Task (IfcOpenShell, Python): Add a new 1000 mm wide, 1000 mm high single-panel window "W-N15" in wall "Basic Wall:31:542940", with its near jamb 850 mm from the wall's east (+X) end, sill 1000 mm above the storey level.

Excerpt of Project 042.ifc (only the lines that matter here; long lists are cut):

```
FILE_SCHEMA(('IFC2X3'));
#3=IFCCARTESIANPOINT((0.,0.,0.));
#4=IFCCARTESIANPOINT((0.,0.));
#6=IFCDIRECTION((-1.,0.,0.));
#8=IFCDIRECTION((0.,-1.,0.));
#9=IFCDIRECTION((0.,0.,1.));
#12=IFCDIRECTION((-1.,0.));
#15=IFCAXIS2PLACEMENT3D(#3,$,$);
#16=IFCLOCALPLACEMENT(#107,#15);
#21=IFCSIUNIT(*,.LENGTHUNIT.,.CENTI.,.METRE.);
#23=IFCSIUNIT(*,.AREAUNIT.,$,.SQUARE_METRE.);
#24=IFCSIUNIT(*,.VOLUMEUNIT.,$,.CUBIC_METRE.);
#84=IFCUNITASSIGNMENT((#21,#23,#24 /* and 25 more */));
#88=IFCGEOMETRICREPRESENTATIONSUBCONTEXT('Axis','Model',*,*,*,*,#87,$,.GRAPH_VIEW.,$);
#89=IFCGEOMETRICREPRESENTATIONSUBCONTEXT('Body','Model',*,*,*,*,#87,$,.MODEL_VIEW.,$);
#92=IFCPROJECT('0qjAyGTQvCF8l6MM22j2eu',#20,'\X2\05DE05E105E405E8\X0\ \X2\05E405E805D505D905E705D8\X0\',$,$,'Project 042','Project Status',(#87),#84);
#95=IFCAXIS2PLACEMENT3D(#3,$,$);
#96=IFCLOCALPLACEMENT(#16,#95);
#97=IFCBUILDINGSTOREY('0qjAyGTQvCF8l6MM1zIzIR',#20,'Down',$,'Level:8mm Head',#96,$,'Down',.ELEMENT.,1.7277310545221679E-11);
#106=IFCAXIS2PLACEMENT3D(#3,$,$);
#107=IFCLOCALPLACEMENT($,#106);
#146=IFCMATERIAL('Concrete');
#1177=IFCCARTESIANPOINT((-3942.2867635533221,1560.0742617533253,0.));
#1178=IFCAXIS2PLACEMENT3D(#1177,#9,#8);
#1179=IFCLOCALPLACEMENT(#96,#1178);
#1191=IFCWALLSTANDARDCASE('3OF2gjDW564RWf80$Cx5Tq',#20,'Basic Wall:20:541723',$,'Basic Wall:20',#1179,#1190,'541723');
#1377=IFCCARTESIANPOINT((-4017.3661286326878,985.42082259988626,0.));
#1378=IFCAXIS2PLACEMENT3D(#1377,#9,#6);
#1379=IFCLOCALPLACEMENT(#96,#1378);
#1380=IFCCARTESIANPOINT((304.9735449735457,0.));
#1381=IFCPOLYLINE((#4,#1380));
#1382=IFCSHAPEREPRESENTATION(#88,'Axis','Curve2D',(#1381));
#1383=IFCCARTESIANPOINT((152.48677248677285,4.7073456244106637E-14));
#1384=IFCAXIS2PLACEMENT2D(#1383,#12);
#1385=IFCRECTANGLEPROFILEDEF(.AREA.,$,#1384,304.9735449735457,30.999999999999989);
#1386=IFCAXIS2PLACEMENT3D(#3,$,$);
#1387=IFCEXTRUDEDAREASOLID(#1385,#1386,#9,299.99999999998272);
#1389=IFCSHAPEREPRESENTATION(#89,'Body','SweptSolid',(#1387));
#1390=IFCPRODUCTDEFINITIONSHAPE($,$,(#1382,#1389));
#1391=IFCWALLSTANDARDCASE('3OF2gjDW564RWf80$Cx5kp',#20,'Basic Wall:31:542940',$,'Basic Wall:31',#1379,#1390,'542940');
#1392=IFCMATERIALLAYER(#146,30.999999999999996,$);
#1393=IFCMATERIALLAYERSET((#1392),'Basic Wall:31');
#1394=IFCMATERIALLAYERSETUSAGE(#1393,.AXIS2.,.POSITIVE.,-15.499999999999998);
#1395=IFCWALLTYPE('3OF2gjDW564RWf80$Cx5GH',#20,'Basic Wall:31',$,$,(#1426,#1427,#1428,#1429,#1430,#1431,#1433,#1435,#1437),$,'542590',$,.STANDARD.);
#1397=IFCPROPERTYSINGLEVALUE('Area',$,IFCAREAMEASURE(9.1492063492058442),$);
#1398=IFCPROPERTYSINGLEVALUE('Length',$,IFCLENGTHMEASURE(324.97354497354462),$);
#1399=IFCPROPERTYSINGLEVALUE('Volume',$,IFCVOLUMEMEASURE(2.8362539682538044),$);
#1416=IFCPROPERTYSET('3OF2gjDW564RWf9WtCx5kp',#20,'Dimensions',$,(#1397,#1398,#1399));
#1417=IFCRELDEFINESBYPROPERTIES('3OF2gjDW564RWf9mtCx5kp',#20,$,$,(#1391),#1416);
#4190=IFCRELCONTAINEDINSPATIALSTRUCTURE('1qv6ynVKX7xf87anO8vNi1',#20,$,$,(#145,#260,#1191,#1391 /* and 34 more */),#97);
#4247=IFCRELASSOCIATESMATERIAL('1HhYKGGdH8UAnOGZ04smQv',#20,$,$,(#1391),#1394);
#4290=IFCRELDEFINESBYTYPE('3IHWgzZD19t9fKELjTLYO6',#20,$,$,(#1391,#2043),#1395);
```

```python
import numpy as np
import ifcopenshell
import ifcopenshell.api.feature
import ifcopenshell.api.geometry
import ifcopenshell.api.pset
import ifcopenshell.api.root
import ifcopenshell.api.spatial
import ifcopenshell.api.type
import ifcopenshell.geom
import ifcopenshell.util.element
import ifcopenshell.util.placement
import ifcopenshell.util.representation
import ifcopenshell.util.shape
import ifcopenshell.util.unit

model = ifcopenshell.open("Project 042.ifc")
unit_scale = ifcopenshell.util.unit.calculate_unit_scale(model)
area_scale = ifcopenshell.util.unit.calculate_unit_scale(model, "AREAUNIT")
volume_scale = ifcopenshell.util.unit.calculate_unit_scale(model, "VOLUMEUNIT")
settings = ifcopenshell.geom.settings()


def volume(element):
    """Net volume in cubic metres, openings subtracted."""
    shape = ifcopenshell.geom.create_shape(settings, element)
    return ifcopenshell.util.shape.get_volume(shape.geometry)


wall = model.by_guid("3OF2gjDW564RWf80$Cx5kp")
storey = ifcopenshell.util.element.get_container(wall, ifc_class="IfcBuildingStorey")
context = ifcopenshell.util.representation.get_context(model, "Model", "Body", "MODEL_VIEW")
before = volume(wall)

width, height, from_end, sill = 1, 1, 0.85, 1  # metres

# The wall runs along its own X axis, and the end named is its -X end.
wall_shape = ifcopenshell.geom.create_shape(settings, wall)
x, y, z = ifcopenshell.util.shape.get_vertices(wall_shape.geometry).T
start = x.min() + from_end
face, thickness = float(y.min()), float(y.max() - y.min())
wall_matrix = ifcopenshell.util.placement.get_local_placement(wall.ObjectPlacement)
level = ifcopenshell.util.placement.get_local_placement(storey.ObjectPlacement)[2, 3]


def in_wall(x, y):
    """Placement at x, y metres in the wall's axes, at sill height."""
    matrix = wall_matrix.copy()
    matrix[:, 3] = wall_matrix @ np.array([x / unit_scale, y / unit_scale, 0.0, 1.0])
    matrix[2, 3] = level + sill / unit_scale
    return matrix


# Opening: a box that overshoots both wall faces by 50 mm.
opening = ifcopenshell.api.root.create_entity(model, ifc_class="IfcOpeningElement")
box = ifcopenshell.api.geometry.add_wall_representation(
    model, context=context, length=width, height=height, thickness=thickness + 0.1
)
ifcopenshell.api.geometry.assign_representation(model, product=opening, representation=box)
ifcopenshell.api.geometry.edit_object_placement(model, product=opening, matrix=in_wall(start, face - 0.05), is_si=False)
ifcopenshell.api.feature.add_feature(model, feature=opening, element=wall)

window = ifcopenshell.api.root.create_entity(model, ifc_class="IfcWindow", name="W-N15")
window.OverallWidth, window.OverallHeight = width / unit_scale, height / unit_scale
body = ifcopenshell.api.geometry.add_window_representation(
    model,
    context=context,
    overall_width=window.OverallWidth,
    overall_height=window.OverallHeight,
    partition_type="SINGLE_PANEL",
)
ifcopenshell.api.geometry.assign_representation(model, product=window, representation=body)
ifcopenshell.api.spatial.assign_container(model, products=[window], relating_structure=storey)
fills = ifcopenshell.api.feature.add_filling(model, opening=opening, element=window)
fills.OwnerHistory = window.OwnerHistory  # required in IFC2X3

# IFC2X3 keeps the operation on the window style.
style = ifcopenshell.api.root.create_entity(model, ifc_class="IfcWindowStyle", name="W-N15")
style.OperationType, style.ConstructionType = "SINGLE_PANEL", "NOTDEFINED"
style.ParameterTakesPrecedence = style.Sizeable = False
ifcopenshell.api.type.assign_type(model, related_objects=[window], relating_type=style)

# Centre the window in the wall's thickness.
ifcopenshell.api.geometry.edit_object_placement(model, product=window, matrix=in_wall(start, face), is_si=False)
window_shape = ifcopenshell.geom.create_shape(settings, window)
depth = ifcopenshell.util.shape.get_vertices(window_shape.geometry)[:, 1]
offset = face + thickness / 2 - (depth.min() + depth.max()) / 2
ifcopenshell.api.geometry.edit_object_placement(model, product=window, matrix=in_wall(start, offset), is_si=False)

after = volume(wall)

# Update the wall's stored quantities.
pset = model.by_id(ifcopenshell.util.element.get_pset(wall, "Dimensions", should_inherit=False)["id"])
ifcopenshell.api.pset.edit_pset(model, pset=pset, properties={
    "Area": model.create_entity("IfcAreaMeasure", after / thickness / area_scale),
    "Volume": model.create_entity("IfcVolumeMeasure", after / volume_scale),
})

print(f"wall volume {before:.3f} -> {after:.3f} m3")

model.write("Project 042-out.ifc")
```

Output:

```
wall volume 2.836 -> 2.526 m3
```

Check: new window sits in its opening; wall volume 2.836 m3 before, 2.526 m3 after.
